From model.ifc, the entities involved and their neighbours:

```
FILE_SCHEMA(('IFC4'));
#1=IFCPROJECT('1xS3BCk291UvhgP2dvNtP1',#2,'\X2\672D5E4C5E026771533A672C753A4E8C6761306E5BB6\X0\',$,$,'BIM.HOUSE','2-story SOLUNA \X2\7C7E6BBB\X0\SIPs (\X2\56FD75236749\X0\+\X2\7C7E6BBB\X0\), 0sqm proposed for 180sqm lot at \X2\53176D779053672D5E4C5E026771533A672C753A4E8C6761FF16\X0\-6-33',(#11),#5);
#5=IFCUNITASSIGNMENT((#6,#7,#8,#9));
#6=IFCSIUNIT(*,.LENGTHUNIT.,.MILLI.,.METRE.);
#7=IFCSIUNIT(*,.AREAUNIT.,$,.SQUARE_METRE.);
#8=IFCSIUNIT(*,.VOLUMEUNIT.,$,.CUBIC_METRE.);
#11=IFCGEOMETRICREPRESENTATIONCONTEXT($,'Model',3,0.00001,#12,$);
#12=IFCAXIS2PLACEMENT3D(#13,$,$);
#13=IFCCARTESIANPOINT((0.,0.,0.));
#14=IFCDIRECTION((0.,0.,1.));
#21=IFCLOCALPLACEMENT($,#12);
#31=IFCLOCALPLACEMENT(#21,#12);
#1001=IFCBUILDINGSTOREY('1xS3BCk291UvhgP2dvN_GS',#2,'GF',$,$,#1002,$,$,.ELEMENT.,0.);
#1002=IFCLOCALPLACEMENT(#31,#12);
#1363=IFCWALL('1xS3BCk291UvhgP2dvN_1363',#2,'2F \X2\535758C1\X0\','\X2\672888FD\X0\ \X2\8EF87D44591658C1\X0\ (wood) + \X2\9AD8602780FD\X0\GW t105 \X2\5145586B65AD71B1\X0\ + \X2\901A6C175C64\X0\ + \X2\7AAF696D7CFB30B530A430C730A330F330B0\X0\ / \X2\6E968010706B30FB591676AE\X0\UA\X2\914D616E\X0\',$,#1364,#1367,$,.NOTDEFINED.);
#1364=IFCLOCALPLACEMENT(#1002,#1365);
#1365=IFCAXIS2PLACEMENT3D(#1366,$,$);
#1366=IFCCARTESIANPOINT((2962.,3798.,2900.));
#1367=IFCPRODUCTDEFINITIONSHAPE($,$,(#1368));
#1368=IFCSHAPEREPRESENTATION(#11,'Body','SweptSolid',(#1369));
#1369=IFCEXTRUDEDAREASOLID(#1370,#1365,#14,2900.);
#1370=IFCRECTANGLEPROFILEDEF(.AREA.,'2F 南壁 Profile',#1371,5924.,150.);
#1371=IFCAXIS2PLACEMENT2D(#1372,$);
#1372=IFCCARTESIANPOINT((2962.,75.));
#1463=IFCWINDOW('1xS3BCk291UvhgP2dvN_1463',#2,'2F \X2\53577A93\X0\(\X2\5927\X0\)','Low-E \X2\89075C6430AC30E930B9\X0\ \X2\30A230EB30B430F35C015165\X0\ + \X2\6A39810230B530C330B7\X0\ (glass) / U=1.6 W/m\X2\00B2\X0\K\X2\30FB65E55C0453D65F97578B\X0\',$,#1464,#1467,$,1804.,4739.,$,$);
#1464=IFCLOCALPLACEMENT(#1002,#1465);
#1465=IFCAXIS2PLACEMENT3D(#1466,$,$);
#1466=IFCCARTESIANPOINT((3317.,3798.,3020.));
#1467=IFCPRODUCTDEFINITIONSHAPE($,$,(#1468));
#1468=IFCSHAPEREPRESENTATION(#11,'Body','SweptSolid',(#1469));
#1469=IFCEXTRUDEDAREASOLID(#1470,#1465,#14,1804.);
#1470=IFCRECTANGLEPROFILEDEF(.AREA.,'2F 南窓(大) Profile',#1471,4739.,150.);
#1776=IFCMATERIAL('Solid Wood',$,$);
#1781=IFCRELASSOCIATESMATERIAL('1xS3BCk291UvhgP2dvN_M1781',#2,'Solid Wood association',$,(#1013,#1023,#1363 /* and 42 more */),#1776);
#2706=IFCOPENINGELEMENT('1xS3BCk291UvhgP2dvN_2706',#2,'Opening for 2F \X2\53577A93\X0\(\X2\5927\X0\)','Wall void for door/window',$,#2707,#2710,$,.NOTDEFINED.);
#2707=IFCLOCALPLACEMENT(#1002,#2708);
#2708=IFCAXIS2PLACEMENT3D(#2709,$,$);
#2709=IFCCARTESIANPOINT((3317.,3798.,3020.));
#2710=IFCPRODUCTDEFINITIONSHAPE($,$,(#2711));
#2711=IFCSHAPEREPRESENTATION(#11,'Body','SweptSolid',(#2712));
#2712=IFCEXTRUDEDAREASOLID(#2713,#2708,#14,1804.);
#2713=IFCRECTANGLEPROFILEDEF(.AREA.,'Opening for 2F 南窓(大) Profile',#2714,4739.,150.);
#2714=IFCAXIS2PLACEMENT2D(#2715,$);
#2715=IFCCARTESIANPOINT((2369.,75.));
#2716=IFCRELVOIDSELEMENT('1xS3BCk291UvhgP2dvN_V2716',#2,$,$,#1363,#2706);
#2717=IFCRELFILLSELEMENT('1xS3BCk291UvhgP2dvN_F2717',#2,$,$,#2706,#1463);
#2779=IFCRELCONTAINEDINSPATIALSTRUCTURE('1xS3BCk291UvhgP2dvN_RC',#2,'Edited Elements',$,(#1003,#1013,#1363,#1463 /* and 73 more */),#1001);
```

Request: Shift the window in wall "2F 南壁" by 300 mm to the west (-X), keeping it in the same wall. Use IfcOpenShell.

```python
import ifcopenshell
import ifcopenshell.api.geometry
import ifcopenshell.util.placement
import ifcopenshell.util.unit

model = ifcopenshell.open("model.ifc")
unit_scale = ifcopenshell.util.unit.calculate_unit_scale(model)

window = model.by_id(1463)
opening = window.FillsVoids[0].RelatingOpeningElement
wall = opening.VoidsElements[0].RelatingBuildingElement

wall_matrix = ifcopenshell.util.placement.get_local_placement(wall.ObjectPlacement)
shift = wall_matrix[:3, 0] * -0.3 / unit_scale
before = ifcopenshell.util.placement.get_local_placement(window.ObjectPlacement)[:3, 3].copy()

# The window is not placed relative to its opening, so move both.
for product in (opening, window):
    matrix = ifcopenshell.util.placement.get_local_placement(product.ObjectPlacement)
    matrix[:3, 3] += shift
    ifcopenshell.api.geometry.edit_object_placement(model, product=product, matrix=matrix, is_si=False)

after = ifcopenshell.util.placement.get_local_placement(window.ObjectPlacement)[:3, 3]
print("window moved by", (after - before).round(3) + 0.0)

model.write("model-out.ifc")
```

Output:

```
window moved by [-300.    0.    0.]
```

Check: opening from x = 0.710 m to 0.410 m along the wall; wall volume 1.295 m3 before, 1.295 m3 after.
